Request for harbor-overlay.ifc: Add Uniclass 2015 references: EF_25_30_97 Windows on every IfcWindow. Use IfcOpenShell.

First a look at what the model holds.

```python
import ifcopenshell

model = ifcopenshell.open("harbor-overlay.ifc")
print(model.schema)
print("classifications:", [c.Name for c in model.by_type("IfcClassification")])
for ifc_class in ("IfcDoor", "IfcRoof", "IfcStair", "IfcWall", "IfcWindow"):
    print(ifc_class, len(model.by_type(ifc_class)))
```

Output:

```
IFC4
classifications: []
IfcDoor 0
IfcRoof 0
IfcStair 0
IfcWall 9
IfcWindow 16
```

```python
import ifcopenshell
import ifcopenshell.api.classification

model = ifcopenshell.open("harbor-overlay.ifc")

system = ifcopenshell.api.classification.add_classification(model, classification="Uniclass 2015")

codes = {
    "IfcWindow": ("EF_25_30_97", "Windows"),
}
for ifc_class, (code, name) in codes.items():
    products = model.by_type(ifc_class)
    ifcopenshell.api.classification.add_reference(
        model, products=products, classification=system, identification=code, name=name
    )
    print(code, len(products))

model.write("harbor-overlay_v2.ifc")
```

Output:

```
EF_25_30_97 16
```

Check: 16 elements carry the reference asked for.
